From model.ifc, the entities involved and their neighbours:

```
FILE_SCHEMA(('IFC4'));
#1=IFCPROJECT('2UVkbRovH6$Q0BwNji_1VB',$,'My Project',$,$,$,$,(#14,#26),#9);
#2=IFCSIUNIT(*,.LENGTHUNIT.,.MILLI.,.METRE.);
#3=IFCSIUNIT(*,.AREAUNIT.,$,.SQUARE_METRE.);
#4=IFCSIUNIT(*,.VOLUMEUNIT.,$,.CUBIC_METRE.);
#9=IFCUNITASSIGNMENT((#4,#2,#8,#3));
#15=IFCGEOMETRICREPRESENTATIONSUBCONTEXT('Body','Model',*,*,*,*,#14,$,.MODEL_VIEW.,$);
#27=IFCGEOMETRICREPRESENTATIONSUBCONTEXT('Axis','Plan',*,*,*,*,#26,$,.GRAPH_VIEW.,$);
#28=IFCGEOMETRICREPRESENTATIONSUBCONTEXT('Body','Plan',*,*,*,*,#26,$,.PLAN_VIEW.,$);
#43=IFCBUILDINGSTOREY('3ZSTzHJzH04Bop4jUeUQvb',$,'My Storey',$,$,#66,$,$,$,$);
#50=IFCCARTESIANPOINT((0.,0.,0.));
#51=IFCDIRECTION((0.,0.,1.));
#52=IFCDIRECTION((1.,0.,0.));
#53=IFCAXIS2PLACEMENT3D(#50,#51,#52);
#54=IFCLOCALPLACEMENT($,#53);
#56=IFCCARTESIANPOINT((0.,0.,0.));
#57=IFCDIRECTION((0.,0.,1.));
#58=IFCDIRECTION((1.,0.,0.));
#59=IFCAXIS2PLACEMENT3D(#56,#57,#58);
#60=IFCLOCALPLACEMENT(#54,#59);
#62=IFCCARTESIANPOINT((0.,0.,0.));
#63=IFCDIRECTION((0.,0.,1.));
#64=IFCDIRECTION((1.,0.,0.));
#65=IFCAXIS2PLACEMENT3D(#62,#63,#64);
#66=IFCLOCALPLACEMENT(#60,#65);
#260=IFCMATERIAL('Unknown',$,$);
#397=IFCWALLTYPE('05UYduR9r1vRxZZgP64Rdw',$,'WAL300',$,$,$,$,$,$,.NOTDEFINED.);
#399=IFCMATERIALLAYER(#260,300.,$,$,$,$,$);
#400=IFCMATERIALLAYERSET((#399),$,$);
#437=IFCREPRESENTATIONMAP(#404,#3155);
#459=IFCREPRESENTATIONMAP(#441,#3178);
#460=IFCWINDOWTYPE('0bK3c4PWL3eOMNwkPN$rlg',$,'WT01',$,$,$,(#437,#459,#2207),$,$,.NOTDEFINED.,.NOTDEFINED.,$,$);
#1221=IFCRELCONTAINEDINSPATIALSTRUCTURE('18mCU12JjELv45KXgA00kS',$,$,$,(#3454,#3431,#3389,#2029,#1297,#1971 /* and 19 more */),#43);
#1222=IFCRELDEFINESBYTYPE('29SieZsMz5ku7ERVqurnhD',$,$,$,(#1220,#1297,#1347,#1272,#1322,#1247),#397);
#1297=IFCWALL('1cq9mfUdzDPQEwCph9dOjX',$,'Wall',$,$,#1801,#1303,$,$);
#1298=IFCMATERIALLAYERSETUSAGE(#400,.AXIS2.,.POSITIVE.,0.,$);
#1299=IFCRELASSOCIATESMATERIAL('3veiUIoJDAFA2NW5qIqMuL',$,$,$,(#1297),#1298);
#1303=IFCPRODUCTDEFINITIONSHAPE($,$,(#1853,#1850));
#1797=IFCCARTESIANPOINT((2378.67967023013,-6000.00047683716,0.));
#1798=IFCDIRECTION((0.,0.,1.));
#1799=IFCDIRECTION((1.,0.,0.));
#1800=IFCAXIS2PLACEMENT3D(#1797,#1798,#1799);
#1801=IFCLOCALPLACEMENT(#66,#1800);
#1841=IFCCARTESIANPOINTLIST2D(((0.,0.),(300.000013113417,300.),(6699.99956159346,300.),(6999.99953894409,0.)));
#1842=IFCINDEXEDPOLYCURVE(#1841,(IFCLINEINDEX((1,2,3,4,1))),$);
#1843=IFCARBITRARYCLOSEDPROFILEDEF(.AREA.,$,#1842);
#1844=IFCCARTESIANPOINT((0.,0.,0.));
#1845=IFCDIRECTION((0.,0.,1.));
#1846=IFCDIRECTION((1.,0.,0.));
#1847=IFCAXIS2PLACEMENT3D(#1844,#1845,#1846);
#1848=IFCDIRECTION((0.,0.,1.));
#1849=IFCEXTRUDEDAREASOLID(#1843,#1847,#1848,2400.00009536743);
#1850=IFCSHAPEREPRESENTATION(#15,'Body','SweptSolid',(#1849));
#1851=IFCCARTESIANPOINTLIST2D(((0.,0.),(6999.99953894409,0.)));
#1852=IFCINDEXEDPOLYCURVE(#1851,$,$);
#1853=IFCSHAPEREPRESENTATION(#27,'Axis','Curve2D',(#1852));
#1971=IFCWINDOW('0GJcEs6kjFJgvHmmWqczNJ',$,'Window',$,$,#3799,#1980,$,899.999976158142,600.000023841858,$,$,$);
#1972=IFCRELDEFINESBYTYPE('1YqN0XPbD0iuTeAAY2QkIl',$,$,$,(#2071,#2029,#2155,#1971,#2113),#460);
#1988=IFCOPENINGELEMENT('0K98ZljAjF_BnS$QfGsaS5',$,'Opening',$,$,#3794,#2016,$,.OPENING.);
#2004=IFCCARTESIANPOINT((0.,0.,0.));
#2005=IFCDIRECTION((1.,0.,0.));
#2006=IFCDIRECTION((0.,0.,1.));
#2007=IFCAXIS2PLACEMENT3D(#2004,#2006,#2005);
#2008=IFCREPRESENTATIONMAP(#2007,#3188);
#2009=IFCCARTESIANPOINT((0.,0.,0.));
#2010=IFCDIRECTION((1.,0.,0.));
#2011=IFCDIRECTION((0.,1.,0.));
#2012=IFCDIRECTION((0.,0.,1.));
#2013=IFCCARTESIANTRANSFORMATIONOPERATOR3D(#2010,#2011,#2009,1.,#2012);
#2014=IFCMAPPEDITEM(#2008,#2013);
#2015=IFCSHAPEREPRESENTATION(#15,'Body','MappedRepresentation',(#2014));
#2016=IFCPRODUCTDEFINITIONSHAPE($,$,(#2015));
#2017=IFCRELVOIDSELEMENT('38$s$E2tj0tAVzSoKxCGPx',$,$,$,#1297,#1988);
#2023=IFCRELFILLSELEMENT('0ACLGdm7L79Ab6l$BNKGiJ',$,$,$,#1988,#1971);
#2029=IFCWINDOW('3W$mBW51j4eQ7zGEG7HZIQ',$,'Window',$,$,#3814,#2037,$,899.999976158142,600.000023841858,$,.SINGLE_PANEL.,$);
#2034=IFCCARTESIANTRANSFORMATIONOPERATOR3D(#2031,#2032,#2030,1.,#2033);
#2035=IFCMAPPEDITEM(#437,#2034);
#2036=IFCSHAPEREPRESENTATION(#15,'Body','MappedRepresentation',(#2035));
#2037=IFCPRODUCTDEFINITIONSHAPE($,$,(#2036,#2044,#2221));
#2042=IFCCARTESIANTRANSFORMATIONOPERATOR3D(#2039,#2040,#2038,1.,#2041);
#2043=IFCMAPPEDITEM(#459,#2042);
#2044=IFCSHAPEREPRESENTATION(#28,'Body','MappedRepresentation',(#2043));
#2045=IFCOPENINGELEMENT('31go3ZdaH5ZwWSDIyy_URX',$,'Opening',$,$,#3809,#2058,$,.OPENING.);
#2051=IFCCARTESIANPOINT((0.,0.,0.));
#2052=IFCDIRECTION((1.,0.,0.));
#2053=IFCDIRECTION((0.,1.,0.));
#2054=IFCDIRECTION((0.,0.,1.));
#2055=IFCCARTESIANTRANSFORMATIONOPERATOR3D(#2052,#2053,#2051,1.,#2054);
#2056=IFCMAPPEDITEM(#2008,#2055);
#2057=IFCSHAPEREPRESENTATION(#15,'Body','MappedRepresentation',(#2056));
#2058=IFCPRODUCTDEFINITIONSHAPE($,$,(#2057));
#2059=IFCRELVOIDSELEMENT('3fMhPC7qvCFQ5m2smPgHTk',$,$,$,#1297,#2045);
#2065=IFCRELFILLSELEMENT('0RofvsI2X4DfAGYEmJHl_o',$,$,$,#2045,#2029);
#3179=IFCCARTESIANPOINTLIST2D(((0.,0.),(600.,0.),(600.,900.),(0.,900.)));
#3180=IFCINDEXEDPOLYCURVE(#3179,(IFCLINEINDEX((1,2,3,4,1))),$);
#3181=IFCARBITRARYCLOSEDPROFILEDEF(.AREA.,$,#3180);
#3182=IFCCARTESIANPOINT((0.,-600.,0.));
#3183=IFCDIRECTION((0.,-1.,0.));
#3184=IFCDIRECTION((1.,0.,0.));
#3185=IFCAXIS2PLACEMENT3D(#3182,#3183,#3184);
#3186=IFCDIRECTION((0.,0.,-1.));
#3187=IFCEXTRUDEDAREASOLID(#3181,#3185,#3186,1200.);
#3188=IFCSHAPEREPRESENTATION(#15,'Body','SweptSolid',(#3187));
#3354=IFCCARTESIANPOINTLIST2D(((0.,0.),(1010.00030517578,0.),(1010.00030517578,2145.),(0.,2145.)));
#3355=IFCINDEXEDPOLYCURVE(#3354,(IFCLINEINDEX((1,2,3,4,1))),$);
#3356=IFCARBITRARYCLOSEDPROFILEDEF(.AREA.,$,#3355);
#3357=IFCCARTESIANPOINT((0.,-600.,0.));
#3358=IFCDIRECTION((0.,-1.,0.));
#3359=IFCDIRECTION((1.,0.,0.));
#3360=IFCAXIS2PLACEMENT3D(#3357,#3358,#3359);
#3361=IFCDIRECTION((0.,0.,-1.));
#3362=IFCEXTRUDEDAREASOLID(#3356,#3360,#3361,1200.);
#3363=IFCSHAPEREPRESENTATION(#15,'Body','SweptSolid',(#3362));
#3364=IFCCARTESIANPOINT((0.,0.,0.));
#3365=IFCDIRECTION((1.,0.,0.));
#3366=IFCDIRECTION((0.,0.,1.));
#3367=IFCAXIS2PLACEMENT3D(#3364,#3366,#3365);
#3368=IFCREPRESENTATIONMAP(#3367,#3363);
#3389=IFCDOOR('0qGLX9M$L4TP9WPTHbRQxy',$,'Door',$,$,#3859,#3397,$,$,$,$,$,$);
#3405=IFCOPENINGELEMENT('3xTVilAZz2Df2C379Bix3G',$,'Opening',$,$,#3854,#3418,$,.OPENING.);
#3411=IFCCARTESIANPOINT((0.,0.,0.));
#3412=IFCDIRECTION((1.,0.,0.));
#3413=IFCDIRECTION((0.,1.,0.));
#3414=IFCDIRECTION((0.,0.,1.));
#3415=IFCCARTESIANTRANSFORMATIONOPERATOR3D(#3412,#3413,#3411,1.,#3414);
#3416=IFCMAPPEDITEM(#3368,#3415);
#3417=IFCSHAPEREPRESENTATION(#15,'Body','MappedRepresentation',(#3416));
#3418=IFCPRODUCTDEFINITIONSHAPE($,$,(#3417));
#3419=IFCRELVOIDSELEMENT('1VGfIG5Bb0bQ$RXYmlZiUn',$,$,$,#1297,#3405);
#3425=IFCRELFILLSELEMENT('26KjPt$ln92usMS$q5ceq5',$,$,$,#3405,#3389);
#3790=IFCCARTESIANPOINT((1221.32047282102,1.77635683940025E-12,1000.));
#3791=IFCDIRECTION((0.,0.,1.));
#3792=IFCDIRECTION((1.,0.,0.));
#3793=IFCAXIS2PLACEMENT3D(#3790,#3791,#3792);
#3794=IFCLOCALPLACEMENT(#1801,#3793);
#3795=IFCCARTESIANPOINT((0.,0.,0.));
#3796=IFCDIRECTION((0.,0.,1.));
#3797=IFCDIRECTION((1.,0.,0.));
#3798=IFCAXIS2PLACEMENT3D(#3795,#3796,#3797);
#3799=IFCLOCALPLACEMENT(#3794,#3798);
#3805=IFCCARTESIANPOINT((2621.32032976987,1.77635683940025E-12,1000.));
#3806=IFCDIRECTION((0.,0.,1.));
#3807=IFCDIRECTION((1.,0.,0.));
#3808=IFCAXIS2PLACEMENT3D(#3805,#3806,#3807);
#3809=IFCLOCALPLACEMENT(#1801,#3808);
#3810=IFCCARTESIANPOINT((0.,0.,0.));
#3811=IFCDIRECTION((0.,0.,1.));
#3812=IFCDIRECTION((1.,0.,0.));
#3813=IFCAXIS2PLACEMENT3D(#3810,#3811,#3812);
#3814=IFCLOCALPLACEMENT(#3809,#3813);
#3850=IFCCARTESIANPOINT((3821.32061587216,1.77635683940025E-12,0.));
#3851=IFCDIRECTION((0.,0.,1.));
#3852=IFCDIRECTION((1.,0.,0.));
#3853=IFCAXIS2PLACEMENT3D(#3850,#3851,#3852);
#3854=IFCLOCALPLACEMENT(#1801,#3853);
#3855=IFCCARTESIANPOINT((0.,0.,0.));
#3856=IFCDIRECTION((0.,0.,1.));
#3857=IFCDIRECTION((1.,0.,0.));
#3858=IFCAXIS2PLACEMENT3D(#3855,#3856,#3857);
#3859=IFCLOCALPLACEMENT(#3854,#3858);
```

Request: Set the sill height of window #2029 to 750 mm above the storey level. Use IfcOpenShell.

```python
import numpy as np
import ifcopenshell
import ifcopenshell.api.geometry
import ifcopenshell.geom
import ifcopenshell.util.element
import ifcopenshell.util.placement
import ifcopenshell.util.shape
import ifcopenshell.util.unit

model = ifcopenshell.open("model.ifc")
unit_scale = ifcopenshell.util.unit.calculate_unit_scale(model)

window = model.by_guid("3W$mBW51j4eQ7zGEG7HZIQ")
opening = window.FillsVoids[0].RelatingOpeningElement
storey = ifcopenshell.util.element.get_container(window, ifc_class="IfcBuildingStorey")
level = ifcopenshell.util.placement.get_local_placement(storey.ObjectPlacement)[2, 3]

# The opening's origin need not be at the sill, so measure its lowest point.
shape = ifcopenshell.geom.create_shape(ifcopenshell.geom.settings(), opening)
bottom = ifcopenshell.util.shape.get_shape_bottom_elevation(shape, shape.geometry) / unit_scale
dz = level + 750.0 - bottom

shift = np.array([0.0, 0.0, dz])
# The window is placed relative to its opening, so it follows when the opening moves.
matrix = ifcopenshell.util.placement.get_local_placement(opening.ObjectPlacement)
matrix[:3, 3] += shift
ifcopenshell.api.geometry.edit_object_placement(
    model, product=opening, matrix=matrix, is_si=False, should_transform_children=True
)

print(f"moved by {dz * unit_scale:+.3f} m")

model.write("model_updated.ifc")
```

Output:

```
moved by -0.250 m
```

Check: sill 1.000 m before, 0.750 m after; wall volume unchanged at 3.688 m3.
